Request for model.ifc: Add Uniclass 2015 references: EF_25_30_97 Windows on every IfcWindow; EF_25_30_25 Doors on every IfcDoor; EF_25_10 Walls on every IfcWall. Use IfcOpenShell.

First a look at what the model holds.

```python
import ifcopenshell

model = ifcopenshell.open("model.ifc")
print(model.schema)
print("classifications:", [c.Name for c in model.by_type("IfcClassification")])
for ifc_class in ("IfcDoor", "IfcRoof", "IfcStair", "IfcWall", "IfcWindow"):
    print(ifc_class, len(model.by_type(ifc_class)))
```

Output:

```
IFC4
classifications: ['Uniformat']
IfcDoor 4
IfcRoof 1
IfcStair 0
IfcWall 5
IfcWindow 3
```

```python
import ifcopenshell
import ifcopenshell.api.classification

model = ifcopenshell.open("model.ifc")

system = ifcopenshell.api.classification.add_classification(model, classification="Uniclass 2015")

codes = {
    "IfcWindow": ("EF_25_30_97", "Windows"),
    "IfcDoor": ("EF_25_30_25", "Doors"),
    "IfcWall": ("EF_25_10", "Walls"),
}
for ifc_class, (code, name) in codes.items():
    products = model.by_type(ifc_class)
    ifcopenshell.api.classification.add_reference(
        model, products=products, classification=system, identification=code, name=name
    )
    print(code, len(products))

model.write("model_rev.ifc")
```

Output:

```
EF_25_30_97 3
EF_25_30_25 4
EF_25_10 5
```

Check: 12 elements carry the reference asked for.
